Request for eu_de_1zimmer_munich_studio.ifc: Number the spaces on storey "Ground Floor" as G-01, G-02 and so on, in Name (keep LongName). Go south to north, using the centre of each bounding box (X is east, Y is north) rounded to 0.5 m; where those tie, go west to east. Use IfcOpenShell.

First a look at what the model holds.

```python
import ifcopenshell
import ifcopenshell.util.element
import ifcopenshell.util.placement

model = ifcopenshell.open("eu_de_1zimmer_munich_studio.ifc")
print(model.schema)
storey = next(s for s in model.by_type("IfcBuildingStorey") if s.Name == "Ground Floor")
spaces = [e for e in ifcopenshell.util.element.get_decomposition(storey) if e.is_a("IfcSpace")]
for e in sorted(spaces, key=lambda e: e.id()):
    origin = ifcopenshell.util.placement.get_local_placement(e.ObjectPlacement)[:3, 3]
    print(e.id(), e.Name, e.LongName, origin.round(2) + 0.0, sep=" | ")
```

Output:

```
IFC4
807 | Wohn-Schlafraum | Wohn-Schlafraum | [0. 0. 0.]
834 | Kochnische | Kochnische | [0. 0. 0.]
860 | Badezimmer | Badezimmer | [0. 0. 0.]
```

```python
import ifcopenshell
import ifcopenshell.geom
import ifcopenshell.util.element
import ifcopenshell.util.shape

model = ifcopenshell.open("eu_de_1zimmer_munich_studio.ifc")
settings = ifcopenshell.geom.settings()
settings.set("use-world-coords", True)


def centre(element):
    shape = ifcopenshell.geom.create_shape(settings, element)
    return ifcopenshell.util.shape.get_bbox_centroid(shape.geometry)


storey = next(s for s in model.by_type("IfcBuildingStorey") if s.Name == "Ground Floor")
spaces = [e for e in ifcopenshell.util.element.get_decomposition(storey) if e.is_a("IfcSpace")]

# Insertion points can sit at a corner or the storey origin, so sort by the geometry (in metres).
centres = {e: centre(e) for e in spaces}
spaces.sort(key=lambda e: (round(centres[e][1] / 0.5), centres[e][0]))

for i, e in enumerate(spaces, start=1):
    number = f"G-{i:02d}"
    e.Name = number
    print(e.id(), number)

model.write("eu_de_1zimmer_munich_studio_edited.ifc")
```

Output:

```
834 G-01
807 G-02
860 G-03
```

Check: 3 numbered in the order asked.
